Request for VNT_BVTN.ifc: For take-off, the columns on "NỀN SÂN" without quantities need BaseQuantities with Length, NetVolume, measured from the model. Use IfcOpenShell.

First a look at what the model holds.

```python
import ifcopenshell
import ifcopenshell.util.element
import ifcopenshell.util.unit

model = ifcopenshell.open("VNT_BVTN.ifc")
print(model.schema)
for unit_type in ("LENGTHUNIT", "AREAUNIT", "VOLUMEUNIT"):
    print(unit_type, ifcopenshell.util.unit.calculate_unit_scale(model, unit_type))
storey = next(s for s in model.by_type("IfcBuildingStorey") if s.Name == "NỀN SÂN")
columns = [e for e in ifcopenshell.util.element.get_decomposition(storey) if e.is_a("IfcColumn")]
for e in sorted(columns, key=lambda e: e.id()):
    print(e.id(), e.is_a(), e.Name, list(ifcopenshell.util.element.get_psets(e, qtos_only=True)), sep=" | ")
```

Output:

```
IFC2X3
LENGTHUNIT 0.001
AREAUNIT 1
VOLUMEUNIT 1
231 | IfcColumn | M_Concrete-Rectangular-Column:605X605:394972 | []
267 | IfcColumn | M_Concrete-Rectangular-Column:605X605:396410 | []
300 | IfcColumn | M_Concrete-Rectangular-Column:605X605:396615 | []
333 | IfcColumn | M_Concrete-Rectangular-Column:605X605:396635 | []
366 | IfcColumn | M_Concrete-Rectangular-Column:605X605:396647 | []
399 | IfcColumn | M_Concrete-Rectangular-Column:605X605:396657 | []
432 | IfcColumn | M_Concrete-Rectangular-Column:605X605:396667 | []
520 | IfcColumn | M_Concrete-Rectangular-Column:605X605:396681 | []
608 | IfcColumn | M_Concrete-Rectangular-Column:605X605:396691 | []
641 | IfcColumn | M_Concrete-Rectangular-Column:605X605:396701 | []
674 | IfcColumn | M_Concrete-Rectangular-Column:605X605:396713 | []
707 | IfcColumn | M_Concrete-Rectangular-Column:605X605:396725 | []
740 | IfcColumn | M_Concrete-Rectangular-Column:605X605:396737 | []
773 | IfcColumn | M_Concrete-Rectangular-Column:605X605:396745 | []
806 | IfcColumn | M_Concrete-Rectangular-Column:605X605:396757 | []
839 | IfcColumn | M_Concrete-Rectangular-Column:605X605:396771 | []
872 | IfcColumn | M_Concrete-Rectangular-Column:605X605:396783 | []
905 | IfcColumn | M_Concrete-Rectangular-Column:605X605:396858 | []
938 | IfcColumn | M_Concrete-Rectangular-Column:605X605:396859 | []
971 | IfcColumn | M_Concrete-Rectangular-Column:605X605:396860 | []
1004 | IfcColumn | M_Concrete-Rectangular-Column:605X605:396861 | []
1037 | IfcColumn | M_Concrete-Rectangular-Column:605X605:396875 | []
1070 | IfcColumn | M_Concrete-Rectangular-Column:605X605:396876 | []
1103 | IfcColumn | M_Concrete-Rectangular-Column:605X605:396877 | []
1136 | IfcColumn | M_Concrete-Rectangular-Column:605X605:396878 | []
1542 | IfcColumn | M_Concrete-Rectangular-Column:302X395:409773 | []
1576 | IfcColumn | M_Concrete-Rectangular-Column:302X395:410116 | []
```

```python
import ifcopenshell
import ifcopenshell.api.pset
import ifcopenshell.geom
import ifcopenshell.util.element
import ifcopenshell.util.shape
import ifcopenshell.util.unit

model = ifcopenshell.open("VNT_BVTN.ifc")
unit_scale = ifcopenshell.util.unit.calculate_unit_scale(model)
volume_scale = ifcopenshell.util.unit.calculate_unit_scale(model, "VOLUMEUNIT")
settings = ifcopenshell.geom.settings()

storey = next(s for s in model.by_type("IfcBuildingStorey") if s.Name == "NỀN SÂN")
columns = [e for e in ifcopenshell.util.element.get_decomposition(storey) if e.is_a("IfcColumn")]

for e in sorted(columns, key=lambda e: e.id()):
    if ifcopenshell.util.element.get_psets(e, qtos_only=True, should_inherit=False):
        continue
    # Geometry comes back in metres, in the element's own axes.
    shape = ifcopenshell.geom.create_shape(settings, e)
    values = {
        "Length": ifcopenshell.util.shape.get_z(shape.geometry) / unit_scale,
        "NetVolume": ifcopenshell.util.shape.get_volume(shape.geometry) / volume_scale,
    }
    qto = ifcopenshell.api.pset.add_qto(model, product=e, name="BaseQuantities")
    ifcopenshell.api.pset.edit_qto(model, qto=qto, properties=values)
    print(e.id(), {k: round(v, 3) for k, v in values.items()})

model.write("VNT_BVTN_edited.ifc")
```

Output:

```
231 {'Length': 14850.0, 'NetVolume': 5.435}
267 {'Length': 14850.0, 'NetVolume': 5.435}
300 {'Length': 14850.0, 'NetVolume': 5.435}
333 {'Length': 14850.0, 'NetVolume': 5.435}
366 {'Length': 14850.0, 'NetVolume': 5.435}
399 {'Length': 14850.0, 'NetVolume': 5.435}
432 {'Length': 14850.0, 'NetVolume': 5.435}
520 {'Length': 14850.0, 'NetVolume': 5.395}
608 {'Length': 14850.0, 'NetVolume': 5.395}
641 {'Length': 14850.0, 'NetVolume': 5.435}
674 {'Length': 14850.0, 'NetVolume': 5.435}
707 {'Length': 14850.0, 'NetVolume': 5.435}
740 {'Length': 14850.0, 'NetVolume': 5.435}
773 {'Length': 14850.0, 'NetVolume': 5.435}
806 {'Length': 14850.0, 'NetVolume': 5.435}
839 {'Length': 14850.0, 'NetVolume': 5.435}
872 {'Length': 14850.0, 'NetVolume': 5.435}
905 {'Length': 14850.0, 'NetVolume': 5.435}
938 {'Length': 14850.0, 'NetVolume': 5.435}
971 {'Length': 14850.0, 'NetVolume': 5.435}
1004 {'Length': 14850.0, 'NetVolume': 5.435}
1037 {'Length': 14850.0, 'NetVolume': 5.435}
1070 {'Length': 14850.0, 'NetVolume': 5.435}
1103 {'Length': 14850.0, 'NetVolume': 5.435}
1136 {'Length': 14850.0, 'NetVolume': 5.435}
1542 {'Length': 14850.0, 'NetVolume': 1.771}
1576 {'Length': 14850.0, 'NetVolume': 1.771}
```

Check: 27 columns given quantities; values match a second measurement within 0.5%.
